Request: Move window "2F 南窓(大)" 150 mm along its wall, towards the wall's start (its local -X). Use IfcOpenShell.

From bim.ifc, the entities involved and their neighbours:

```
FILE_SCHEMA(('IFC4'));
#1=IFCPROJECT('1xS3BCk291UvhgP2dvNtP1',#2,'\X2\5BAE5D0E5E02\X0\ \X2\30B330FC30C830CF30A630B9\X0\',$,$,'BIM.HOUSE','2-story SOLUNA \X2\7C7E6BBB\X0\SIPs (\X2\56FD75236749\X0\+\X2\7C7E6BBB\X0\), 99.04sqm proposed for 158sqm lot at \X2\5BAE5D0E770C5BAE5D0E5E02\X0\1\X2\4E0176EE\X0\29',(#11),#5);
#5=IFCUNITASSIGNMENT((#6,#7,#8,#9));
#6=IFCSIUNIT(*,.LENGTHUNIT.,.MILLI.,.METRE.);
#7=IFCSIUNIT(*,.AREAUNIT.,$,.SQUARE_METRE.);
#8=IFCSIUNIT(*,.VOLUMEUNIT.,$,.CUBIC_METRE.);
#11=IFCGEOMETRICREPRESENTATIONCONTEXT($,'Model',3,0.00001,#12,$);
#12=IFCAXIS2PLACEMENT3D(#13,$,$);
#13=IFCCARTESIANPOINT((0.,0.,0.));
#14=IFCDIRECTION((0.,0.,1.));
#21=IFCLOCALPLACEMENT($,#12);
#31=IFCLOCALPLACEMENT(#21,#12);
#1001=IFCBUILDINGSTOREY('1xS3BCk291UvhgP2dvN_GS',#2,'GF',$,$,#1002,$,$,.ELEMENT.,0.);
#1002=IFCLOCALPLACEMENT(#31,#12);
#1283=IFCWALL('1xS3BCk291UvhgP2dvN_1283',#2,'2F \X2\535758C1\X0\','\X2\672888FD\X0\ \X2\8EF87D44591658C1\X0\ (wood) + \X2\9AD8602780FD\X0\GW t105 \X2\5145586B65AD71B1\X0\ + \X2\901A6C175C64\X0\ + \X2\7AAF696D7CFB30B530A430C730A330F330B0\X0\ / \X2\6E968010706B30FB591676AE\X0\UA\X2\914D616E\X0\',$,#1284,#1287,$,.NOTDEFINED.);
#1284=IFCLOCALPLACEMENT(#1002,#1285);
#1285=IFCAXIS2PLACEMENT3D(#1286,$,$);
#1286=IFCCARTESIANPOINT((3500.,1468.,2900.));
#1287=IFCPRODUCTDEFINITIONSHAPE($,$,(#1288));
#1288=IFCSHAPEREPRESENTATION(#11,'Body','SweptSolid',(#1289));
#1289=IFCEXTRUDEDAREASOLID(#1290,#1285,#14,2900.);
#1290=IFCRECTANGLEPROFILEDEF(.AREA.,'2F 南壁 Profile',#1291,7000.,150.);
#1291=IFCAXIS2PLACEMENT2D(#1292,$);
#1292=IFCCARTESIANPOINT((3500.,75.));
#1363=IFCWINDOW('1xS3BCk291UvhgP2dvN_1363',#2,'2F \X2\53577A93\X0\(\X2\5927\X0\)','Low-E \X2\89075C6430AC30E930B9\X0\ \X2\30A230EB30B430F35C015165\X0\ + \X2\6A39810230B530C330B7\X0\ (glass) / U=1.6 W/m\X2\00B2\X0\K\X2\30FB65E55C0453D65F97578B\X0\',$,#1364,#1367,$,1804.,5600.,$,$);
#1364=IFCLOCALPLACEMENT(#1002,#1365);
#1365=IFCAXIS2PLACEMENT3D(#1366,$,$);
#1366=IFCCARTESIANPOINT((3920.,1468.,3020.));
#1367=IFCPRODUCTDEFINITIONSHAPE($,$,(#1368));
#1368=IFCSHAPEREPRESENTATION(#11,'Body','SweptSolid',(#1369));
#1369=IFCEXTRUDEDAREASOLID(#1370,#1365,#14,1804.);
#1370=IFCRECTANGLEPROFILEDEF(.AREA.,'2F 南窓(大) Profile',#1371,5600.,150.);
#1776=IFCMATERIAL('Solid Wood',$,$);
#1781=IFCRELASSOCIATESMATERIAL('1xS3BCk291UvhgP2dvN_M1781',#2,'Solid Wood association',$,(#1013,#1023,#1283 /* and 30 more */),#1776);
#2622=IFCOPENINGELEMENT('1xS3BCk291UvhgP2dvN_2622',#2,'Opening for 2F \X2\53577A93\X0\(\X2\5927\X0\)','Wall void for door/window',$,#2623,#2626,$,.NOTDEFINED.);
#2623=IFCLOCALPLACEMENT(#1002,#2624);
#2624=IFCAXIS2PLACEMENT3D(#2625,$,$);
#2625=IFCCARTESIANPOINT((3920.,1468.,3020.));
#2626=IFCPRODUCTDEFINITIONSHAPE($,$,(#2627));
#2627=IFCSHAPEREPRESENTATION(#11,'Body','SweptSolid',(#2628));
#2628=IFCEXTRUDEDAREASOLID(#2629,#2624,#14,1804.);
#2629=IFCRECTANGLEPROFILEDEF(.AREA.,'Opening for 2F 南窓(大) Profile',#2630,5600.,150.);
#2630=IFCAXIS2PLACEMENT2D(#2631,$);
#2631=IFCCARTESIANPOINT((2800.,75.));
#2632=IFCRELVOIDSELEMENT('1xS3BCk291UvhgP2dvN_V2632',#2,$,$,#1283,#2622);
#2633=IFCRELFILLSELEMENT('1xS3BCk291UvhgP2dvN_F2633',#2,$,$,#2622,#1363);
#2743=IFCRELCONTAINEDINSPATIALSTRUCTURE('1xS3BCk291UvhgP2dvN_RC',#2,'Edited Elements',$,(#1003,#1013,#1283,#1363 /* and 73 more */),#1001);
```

```python
import ifcopenshell
import ifcopenshell.api.geometry
import ifcopenshell.util.placement
import ifcopenshell.util.unit

model = ifcopenshell.open("bim.ifc")
unit_scale = ifcopenshell.util.unit.calculate_unit_scale(model)

window = model.by_guid("1xS3BCk291UvhgP2dvN_1363")
opening = window.FillsVoids[0].RelatingOpeningElement
wall = opening.VoidsElements[0].RelatingBuildingElement

wall_matrix = ifcopenshell.util.placement.get_local_placement(wall.ObjectPlacement)
shift = wall_matrix[:3, 0] * -0.15 / unit_scale
before = ifcopenshell.util.placement.get_local_placement(window.ObjectPlacement)[:3, 3].copy()

# The window is not placed relative to its opening, so move both.
for product in (opening, window):
    matrix = ifcopenshell.util.placement.get_local_placement(product.ObjectPlacement)
    matrix[:3, 3] += shift
    ifcopenshell.api.geometry.edit_object_placement(model, product=product, matrix=matrix, is_si=False)

after = ifcopenshell.util.placement.get_local_placement(window.ObjectPlacement)[:3, 3]
print("window moved by", (after - before).round(3) + 0.0)

model.write("bim-out.ifc")
```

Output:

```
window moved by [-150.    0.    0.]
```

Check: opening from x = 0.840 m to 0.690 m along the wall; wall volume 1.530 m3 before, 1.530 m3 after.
